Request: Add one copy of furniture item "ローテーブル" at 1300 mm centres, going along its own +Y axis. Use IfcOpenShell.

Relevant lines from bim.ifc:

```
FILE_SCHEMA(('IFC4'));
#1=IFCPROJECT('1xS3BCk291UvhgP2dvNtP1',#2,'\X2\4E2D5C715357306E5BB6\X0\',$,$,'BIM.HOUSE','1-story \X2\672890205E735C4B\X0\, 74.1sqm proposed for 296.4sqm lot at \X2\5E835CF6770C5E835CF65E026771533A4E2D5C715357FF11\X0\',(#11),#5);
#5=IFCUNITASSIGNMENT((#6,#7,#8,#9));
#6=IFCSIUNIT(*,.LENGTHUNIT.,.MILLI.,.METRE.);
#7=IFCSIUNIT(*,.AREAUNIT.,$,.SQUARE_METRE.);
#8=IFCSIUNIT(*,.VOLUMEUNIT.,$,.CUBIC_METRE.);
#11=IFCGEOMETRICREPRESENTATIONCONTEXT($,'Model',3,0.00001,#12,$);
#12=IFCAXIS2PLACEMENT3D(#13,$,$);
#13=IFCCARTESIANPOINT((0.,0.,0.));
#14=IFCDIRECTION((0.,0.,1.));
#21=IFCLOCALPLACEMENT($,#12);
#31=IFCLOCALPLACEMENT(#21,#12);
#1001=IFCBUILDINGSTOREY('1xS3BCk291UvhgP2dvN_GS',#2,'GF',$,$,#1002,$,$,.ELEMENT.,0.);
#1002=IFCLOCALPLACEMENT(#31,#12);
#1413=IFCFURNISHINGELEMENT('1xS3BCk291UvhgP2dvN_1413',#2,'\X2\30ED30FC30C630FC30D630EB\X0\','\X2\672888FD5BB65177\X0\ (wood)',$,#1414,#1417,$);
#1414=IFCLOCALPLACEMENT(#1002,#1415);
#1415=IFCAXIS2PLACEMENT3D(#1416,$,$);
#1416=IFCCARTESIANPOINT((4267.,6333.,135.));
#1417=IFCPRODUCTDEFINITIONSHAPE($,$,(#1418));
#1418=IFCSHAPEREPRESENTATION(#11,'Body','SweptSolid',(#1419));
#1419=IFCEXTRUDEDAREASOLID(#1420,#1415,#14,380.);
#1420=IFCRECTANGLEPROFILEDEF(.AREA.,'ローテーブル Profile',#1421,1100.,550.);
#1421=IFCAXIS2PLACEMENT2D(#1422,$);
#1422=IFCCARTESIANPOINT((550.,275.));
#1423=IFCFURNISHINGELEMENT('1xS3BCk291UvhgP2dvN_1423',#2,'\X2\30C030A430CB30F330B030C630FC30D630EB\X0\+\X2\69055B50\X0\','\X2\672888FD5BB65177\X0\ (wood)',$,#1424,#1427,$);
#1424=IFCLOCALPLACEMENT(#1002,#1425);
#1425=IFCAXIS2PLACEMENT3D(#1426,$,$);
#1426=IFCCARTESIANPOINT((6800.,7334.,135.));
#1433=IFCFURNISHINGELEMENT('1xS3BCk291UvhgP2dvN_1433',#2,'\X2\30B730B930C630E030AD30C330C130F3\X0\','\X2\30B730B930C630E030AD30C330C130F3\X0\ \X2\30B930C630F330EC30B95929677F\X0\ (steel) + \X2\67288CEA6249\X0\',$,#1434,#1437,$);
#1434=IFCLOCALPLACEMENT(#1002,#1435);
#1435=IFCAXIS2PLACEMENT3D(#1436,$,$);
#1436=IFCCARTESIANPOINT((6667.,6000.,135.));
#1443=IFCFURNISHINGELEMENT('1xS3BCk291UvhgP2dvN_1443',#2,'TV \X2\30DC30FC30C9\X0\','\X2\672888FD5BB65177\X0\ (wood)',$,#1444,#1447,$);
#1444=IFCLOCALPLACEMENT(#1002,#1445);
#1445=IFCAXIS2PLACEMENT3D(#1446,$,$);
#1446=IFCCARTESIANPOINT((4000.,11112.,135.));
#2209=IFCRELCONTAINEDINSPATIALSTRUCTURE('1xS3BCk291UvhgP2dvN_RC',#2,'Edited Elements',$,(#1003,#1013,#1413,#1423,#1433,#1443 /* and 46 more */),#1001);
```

```python
import ifcopenshell
import ifcopenshell.api.geometry
import ifcopenshell.api.root
import ifcopenshell.util.element
import ifcopenshell.util.placement

model = ifcopenshell.open("bim.ifc")


def reuse_history(source, copy):
    """copy_class also copies each property set's owner history, people and application; keep the originals."""
    for rel in copy.IsDefinedBy:
        if rel.is_a("IfcRelDefinesByProperties") and (history := rel.RelatingPropertyDefinition.OwnerHistory):
            rel.RelatingPropertyDefinition.OwnerHistory = source.OwnerHistory
            ifcopenshell.util.element.remove_deep2(model, history)


source = model.by_id(1413)
base = ifcopenshell.util.placement.get_local_placement(source.ObjectPlacement)
step = base[:3, 1] * 1300.0

for i in range(1, 2):
    copy = ifcopenshell.api.root.copy_class(model, product=source)
    copy.Representation = ifcopenshell.util.element.copy_deep(
        model, source.Representation, exclude=["IfcGeometricRepresentationContext", "IfcRepresentationMap"]
    )
    reuse_history(source, copy)
    matrix = base.copy()
    matrix[:3, 3] += i * step
    print("added at", matrix[:3, 3].round(3) + 0.0)
    ifcopenshell.api.geometry.edit_object_placement(model, product=copy, matrix=matrix, is_si=False)

model.write("bim_v2.ifc")
```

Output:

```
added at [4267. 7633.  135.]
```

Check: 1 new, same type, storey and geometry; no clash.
